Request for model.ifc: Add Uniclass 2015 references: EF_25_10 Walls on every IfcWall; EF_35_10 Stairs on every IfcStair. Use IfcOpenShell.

First a look at what the model holds.

```python
import ifcopenshell

model = ifcopenshell.open("model.ifc")
print(model.schema)
print("classifications:", [c.Name for c in model.by_type("IfcClassification")])
for ifc_class in ("IfcDoor", "IfcRoof", "IfcStair", "IfcWall", "IfcWindow"):
    print(ifc_class, len(model.by_type(ifc_class)))
```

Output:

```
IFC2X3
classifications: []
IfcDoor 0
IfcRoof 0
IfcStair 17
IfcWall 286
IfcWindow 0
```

```python
import ifcopenshell
import ifcopenshell.api.classification

model = ifcopenshell.open("model.ifc")

# IFC2X3 requires Source and Edition and has no link from the project to the system.
system = model.create_entity("IfcClassification", Source="NBS", Edition="2015", Name="Uniclass 2015")

codes = {
    "IfcWall": ("EF_25_10", "Walls"),
    "IfcStair": ("EF_35_10", "Stairs"),
}
for ifc_class, (code, name) in codes.items():
    products = model.by_type(ifc_class)
    ifcopenshell.api.classification.add_reference(
        model, products=products, classification=system, identification=code, name=name
    )
    print(code, len(products))

model.write("model_rev.ifc")
```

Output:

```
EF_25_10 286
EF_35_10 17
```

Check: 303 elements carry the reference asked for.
